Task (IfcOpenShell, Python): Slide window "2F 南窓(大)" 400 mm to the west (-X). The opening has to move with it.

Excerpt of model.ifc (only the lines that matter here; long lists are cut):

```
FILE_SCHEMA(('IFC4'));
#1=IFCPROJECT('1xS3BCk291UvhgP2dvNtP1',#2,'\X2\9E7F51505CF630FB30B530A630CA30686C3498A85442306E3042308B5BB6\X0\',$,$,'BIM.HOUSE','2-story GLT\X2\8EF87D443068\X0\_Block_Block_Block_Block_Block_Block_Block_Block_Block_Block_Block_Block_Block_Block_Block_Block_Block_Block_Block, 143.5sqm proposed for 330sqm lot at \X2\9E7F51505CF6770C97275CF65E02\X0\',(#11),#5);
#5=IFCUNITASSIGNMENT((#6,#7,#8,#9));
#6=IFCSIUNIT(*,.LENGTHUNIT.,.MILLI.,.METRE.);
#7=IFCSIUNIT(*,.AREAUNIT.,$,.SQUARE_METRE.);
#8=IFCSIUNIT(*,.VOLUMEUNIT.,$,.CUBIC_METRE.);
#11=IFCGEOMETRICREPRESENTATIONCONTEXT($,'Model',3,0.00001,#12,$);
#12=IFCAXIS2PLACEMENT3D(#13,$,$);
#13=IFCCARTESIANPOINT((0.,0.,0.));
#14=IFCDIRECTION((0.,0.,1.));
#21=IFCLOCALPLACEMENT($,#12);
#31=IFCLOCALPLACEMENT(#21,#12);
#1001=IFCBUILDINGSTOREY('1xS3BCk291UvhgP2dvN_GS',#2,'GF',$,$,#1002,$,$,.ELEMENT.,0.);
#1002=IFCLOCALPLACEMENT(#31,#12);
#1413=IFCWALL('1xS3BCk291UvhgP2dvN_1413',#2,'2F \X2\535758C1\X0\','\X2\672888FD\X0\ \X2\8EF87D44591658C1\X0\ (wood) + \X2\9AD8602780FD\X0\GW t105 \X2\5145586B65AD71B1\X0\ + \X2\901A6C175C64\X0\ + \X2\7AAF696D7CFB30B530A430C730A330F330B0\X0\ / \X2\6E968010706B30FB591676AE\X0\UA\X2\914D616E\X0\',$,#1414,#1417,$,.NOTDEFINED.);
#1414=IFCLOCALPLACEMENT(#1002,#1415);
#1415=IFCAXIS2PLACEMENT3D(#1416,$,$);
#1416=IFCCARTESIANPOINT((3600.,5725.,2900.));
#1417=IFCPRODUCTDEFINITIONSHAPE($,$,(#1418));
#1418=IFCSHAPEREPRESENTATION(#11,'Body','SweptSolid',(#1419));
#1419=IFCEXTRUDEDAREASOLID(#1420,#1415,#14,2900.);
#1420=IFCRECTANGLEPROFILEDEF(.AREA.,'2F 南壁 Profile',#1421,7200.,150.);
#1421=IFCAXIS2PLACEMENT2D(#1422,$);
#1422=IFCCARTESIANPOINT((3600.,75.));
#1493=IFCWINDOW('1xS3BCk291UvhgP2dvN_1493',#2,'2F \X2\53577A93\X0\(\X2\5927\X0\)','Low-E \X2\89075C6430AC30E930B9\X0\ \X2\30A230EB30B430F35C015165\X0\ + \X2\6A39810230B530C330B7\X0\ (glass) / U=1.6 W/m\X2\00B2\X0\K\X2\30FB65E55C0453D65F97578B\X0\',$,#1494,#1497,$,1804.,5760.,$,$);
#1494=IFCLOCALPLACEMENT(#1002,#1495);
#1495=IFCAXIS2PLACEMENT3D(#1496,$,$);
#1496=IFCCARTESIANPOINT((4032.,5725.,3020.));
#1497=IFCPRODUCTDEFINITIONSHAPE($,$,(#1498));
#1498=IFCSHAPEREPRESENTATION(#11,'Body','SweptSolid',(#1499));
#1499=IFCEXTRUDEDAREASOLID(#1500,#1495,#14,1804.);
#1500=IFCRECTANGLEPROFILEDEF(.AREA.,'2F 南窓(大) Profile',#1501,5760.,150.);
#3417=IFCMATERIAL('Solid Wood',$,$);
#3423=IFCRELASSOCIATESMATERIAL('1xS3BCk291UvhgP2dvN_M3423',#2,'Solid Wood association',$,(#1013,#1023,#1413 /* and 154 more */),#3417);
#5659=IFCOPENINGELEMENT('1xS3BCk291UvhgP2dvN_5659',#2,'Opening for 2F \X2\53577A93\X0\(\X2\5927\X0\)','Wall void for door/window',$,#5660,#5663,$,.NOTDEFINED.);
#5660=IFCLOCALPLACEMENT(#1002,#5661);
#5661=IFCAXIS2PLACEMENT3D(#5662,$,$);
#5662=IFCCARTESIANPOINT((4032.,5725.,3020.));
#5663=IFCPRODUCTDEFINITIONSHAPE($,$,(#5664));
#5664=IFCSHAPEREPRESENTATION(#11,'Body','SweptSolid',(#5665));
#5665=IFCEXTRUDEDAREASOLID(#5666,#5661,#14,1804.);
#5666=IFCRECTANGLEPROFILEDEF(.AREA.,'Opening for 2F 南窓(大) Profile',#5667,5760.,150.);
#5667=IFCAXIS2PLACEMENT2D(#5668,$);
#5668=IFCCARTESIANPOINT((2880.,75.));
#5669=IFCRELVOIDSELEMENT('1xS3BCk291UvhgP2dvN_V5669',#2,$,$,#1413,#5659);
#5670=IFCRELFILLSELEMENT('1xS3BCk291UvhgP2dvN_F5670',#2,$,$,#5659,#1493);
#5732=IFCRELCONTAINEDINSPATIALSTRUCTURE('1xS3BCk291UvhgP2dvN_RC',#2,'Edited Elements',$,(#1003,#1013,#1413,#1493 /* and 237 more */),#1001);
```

```python
import ifcopenshell
import ifcopenshell.api.geometry
import ifcopenshell.util.placement
import ifcopenshell.util.unit

model = ifcopenshell.open("model.ifc")
unit_scale = ifcopenshell.util.unit.calculate_unit_scale(model)

window = model.by_id(1493)
opening = window.FillsVoids[0].RelatingOpeningElement
wall = opening.VoidsElements[0].RelatingBuildingElement

wall_matrix = ifcopenshell.util.placement.get_local_placement(wall.ObjectPlacement)
shift = wall_matrix[:3, 0] * -0.4 / unit_scale
before = ifcopenshell.util.placement.get_local_placement(window.ObjectPlacement)[:3, 3].copy()

# The window is not placed relative to its opening, so move both.
for product in (opening, window):
    matrix = ifcopenshell.util.placement.get_local_placement(product.ObjectPlacement)
    matrix[:3, 3] += shift
    ifcopenshell.api.geometry.edit_object_placement(model, product=product, matrix=matrix, is_si=False)

after = ifcopenshell.util.placement.get_local_placement(window.ObjectPlacement)[:3, 3]
print("window moved by", (after - before).round(3) + 0.0)

model.write("model_updated.ifc")
```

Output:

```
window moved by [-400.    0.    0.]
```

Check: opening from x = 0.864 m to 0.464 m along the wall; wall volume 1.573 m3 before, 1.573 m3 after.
